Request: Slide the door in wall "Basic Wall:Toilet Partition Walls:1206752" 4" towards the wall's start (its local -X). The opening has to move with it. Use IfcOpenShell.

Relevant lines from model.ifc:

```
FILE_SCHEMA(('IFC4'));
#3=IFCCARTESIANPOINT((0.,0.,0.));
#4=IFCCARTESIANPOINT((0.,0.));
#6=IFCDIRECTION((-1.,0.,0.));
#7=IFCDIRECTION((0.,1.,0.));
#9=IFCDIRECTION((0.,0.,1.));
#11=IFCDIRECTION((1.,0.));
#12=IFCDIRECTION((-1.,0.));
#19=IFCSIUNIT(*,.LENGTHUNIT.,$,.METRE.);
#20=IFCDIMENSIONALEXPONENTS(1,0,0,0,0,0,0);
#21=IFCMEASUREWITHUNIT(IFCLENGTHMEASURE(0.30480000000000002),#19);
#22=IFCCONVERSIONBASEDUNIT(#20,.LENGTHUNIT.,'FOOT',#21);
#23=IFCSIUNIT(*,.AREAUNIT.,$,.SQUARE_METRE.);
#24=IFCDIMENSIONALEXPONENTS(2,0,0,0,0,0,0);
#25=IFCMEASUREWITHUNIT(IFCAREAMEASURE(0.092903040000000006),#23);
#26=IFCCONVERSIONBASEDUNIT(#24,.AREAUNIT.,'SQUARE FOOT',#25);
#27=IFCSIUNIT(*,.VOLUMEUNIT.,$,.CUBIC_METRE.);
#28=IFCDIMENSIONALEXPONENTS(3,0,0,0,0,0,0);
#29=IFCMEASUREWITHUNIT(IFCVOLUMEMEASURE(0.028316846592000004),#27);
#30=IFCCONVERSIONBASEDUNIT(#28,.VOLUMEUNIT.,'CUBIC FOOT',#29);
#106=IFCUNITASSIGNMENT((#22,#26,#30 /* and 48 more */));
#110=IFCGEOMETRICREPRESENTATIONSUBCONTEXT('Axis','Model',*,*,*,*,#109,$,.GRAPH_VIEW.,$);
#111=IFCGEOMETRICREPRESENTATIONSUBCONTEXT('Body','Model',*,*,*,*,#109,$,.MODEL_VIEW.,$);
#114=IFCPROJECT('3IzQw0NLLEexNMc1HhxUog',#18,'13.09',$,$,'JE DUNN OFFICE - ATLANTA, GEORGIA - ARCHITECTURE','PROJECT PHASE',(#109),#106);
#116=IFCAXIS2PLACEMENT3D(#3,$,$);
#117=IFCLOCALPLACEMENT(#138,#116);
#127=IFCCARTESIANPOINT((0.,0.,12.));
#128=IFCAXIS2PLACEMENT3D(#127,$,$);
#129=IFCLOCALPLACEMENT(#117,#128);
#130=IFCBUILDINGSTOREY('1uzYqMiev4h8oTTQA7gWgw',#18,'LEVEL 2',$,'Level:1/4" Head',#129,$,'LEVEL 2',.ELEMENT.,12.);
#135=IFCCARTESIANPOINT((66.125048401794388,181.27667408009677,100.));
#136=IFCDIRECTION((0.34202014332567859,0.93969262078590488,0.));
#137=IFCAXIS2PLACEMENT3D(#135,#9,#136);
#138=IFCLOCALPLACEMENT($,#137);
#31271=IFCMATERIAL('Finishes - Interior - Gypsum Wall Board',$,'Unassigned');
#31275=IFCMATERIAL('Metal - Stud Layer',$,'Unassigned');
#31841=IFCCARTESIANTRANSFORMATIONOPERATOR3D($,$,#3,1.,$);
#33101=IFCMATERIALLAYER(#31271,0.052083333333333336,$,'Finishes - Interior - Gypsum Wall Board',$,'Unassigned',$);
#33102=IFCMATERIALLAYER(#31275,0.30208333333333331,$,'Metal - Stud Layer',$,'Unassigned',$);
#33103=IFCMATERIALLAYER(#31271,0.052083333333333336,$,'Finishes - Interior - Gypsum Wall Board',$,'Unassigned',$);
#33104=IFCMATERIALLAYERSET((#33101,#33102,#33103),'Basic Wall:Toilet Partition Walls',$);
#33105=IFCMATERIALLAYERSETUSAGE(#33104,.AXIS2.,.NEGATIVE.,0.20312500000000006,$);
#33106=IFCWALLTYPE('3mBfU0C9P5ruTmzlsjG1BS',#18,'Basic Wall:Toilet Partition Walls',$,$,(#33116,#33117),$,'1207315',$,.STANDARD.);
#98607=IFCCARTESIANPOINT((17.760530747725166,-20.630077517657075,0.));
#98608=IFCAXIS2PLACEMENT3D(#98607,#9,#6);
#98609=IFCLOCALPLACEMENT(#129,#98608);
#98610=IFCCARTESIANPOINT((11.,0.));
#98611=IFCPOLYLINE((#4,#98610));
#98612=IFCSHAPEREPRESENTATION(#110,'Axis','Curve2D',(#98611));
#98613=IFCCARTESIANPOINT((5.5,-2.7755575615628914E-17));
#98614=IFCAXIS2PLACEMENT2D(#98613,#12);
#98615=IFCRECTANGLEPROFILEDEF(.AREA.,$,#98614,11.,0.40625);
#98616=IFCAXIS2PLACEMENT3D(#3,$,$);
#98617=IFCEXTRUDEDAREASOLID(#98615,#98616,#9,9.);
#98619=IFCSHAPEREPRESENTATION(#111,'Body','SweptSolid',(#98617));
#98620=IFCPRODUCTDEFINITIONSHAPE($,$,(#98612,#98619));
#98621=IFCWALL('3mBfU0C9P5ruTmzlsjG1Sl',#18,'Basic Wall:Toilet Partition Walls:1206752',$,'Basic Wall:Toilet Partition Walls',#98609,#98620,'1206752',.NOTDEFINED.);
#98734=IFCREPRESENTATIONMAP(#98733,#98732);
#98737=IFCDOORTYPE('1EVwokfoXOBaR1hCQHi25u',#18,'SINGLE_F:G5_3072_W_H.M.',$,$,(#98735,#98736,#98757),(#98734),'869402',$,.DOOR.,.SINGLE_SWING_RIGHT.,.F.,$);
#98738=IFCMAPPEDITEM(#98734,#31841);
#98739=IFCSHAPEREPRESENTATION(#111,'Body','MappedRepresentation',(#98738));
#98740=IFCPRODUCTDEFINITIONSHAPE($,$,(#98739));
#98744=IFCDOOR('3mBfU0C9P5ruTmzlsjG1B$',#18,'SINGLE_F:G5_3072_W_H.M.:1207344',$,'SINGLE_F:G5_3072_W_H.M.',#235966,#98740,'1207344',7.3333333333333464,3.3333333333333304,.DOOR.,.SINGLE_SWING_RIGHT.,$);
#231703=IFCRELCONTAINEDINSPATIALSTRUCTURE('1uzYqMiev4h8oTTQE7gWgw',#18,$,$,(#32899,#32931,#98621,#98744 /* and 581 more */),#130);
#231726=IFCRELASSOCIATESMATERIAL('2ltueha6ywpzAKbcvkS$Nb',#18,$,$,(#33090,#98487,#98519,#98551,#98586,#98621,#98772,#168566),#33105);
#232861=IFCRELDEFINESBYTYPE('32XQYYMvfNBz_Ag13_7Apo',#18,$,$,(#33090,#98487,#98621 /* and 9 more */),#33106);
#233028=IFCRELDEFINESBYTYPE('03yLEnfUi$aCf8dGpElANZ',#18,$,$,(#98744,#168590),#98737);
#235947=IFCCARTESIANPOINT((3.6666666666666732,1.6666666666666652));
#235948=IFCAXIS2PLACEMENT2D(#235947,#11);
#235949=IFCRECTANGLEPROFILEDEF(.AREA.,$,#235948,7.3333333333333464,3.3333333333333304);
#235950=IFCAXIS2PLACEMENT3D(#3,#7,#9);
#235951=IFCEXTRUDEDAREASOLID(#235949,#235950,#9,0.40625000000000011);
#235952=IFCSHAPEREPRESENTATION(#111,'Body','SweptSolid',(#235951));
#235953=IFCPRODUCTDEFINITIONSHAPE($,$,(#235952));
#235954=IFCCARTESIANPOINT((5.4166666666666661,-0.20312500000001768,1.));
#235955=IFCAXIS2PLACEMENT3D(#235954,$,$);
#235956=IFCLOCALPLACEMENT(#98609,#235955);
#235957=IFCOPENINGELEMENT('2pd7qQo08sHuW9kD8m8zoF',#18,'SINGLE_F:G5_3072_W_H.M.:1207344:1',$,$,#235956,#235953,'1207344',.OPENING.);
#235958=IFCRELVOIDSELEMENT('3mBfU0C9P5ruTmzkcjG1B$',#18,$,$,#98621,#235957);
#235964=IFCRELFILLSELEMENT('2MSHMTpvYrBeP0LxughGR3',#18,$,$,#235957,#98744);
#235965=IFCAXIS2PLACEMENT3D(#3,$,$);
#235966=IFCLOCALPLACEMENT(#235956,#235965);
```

```python
import ifcopenshell
import ifcopenshell.api.geometry
import ifcopenshell.util.placement
import ifcopenshell.util.unit

model = ifcopenshell.open("model.ifc")
unit_scale = ifcopenshell.util.unit.calculate_unit_scale(model)

door = model.by_guid("3mBfU0C9P5ruTmzlsjG1B$")
opening = door.FillsVoids[0].RelatingOpeningElement
wall = opening.VoidsElements[0].RelatingBuildingElement

wall_matrix = ifcopenshell.util.placement.get_local_placement(wall.ObjectPlacement)
shift = wall_matrix[:3, 0] * -4 * 0.0254 / unit_scale
before = ifcopenshell.util.placement.get_local_placement(door.ObjectPlacement)[:3, 3].copy()

# The door is placed relative to its opening, so it follows when the opening moves.
matrix = ifcopenshell.util.placement.get_local_placement(opening.ObjectPlacement)
matrix[:3, 3] += shift
ifcopenshell.api.geometry.edit_object_placement(
    model, product=opening, matrix=matrix, is_si=False, should_transform_children=True
)

after = ifcopenshell.util.placement.get_local_placement(door.ObjectPlacement)[:3, 3]
print("door moved by", (after - before).round(3) + 0.0)

model.write("model_v2.ifc")
```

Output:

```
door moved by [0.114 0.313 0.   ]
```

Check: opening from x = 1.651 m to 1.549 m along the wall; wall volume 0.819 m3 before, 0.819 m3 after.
